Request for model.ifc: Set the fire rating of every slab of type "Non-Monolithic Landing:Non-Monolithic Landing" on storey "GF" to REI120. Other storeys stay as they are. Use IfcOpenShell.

First a look at what the model holds.

```python
import ifcopenshell
import ifcopenshell.util.element

model = ifcopenshell.open("model.ifc")
print(model.schema)
storey = next(s for s in model.by_type("IfcBuildingStorey") if s.Name == "GF")
slabs = [e for e in ifcopenshell.util.element.get_decomposition(storey) if e.is_a("IfcSlab")]
seen = {}
for e in slabs:
    element_type = ifcopenshell.util.element.get_type(e)
    key = (element_type.Name if element_type != e and element_type else None, ifcopenshell.util.element.get_pset(e, "Pset_SlabCommon", "FireRating"))
    seen[key] = seen.get(key, 0) + 1
for (name, value), count in sorted(seen.items(), key=str):
    print(count, "x", name, "|", value)
```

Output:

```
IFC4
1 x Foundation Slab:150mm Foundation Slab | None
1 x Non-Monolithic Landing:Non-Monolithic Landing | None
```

```python
import ifcopenshell
import ifcopenshell.api.pset
import ifcopenshell.util.element

model = ifcopenshell.open("model.ifc")

storey = next(s for s in model.by_type("IfcBuildingStorey") if s.Name == "GF")
slabs = [e for e in ifcopenshell.util.element.get_decomposition(storey) if e.is_a("IfcSlab")]

count = 0
for e in slabs:
    element_type = ifcopenshell.util.element.get_type(e)
    if element_type in (None, e) or element_type.Name != "Non-Monolithic Landing:Non-Monolithic Landing":
        continue
    # add_pset returns the element's existing set when there is one.
    pset = ifcopenshell.api.pset.add_pset(model, product=e, name="Pset_SlabCommon")
    ifcopenshell.api.pset.edit_pset(model, pset=pset, properties={"FireRating": "REI120"})
    count += 1

print(count, "slabs updated")

model.write("model_edited.ifc")
```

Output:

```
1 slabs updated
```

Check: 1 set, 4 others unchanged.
